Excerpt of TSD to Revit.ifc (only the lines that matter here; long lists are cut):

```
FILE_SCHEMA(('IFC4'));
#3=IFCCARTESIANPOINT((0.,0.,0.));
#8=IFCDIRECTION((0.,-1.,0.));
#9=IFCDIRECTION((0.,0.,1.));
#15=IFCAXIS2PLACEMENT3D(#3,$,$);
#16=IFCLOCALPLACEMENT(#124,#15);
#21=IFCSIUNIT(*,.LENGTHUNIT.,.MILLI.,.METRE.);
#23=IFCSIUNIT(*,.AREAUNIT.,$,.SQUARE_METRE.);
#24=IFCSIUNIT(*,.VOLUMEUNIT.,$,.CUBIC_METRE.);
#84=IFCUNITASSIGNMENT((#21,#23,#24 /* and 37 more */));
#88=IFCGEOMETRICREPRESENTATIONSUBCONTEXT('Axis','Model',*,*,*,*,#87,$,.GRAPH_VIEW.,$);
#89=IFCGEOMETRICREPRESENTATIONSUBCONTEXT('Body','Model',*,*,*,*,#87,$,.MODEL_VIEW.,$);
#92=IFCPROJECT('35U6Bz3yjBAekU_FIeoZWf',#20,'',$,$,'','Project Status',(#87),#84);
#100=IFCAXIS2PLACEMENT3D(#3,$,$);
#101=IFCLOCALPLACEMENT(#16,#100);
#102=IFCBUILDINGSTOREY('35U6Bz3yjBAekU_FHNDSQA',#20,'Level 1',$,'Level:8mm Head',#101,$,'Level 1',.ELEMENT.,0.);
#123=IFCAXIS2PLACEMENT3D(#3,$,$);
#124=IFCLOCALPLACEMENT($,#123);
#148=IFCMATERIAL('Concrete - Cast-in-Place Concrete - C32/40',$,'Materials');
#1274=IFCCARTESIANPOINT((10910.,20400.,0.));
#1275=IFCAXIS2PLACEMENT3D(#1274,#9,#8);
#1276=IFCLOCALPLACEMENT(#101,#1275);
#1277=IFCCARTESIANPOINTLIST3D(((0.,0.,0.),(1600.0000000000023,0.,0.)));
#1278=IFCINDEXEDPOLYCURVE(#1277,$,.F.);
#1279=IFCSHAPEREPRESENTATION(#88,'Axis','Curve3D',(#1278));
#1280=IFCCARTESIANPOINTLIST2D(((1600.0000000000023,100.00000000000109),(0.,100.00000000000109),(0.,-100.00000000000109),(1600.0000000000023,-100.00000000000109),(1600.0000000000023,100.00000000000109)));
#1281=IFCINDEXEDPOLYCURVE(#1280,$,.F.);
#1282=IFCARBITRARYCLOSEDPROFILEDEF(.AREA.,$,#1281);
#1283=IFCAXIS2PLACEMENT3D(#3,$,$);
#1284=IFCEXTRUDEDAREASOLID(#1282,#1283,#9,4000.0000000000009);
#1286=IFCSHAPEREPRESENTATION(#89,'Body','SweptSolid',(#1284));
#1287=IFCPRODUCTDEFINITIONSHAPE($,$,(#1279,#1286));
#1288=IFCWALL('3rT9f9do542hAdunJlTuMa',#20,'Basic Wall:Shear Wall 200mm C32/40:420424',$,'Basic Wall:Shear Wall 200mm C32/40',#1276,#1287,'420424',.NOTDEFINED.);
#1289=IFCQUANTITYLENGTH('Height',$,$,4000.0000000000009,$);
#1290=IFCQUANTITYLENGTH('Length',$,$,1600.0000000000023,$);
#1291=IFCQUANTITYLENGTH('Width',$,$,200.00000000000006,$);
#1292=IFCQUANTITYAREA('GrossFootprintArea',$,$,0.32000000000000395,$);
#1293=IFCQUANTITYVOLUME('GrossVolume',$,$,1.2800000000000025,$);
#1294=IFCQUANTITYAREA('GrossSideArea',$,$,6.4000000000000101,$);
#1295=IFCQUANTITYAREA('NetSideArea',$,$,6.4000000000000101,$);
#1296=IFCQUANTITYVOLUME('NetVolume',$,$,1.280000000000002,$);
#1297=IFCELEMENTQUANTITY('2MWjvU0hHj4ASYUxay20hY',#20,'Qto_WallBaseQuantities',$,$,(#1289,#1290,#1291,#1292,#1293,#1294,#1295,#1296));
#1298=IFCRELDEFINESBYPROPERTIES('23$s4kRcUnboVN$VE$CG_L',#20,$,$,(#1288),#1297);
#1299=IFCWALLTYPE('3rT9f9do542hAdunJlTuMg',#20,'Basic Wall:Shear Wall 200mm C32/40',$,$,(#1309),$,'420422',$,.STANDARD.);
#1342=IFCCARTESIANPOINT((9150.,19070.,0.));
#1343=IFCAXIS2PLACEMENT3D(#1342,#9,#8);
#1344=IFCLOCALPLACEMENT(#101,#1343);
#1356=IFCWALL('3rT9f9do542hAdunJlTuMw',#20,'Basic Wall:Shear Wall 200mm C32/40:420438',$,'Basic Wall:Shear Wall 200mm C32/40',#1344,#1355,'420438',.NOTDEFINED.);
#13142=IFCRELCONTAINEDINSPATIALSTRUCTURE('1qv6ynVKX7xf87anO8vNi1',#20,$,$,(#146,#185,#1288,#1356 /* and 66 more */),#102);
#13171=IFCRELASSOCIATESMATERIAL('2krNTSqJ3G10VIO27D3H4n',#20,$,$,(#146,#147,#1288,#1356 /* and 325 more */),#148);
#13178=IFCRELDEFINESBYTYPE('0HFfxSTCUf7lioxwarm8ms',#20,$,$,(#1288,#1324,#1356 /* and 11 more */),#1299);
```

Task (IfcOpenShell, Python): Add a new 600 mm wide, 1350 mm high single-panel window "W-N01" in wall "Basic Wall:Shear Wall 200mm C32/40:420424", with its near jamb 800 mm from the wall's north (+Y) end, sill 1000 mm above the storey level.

```python
import numpy as np
import ifcopenshell
import ifcopenshell.api.feature
import ifcopenshell.api.geometry
import ifcopenshell.api.pset
import ifcopenshell.api.root
import ifcopenshell.api.spatial
import ifcopenshell.geom
import ifcopenshell.util.element
import ifcopenshell.util.placement
import ifcopenshell.util.representation
import ifcopenshell.util.shape
import ifcopenshell.util.unit

model = ifcopenshell.open("TSD to Revit.ifc")
unit_scale = ifcopenshell.util.unit.calculate_unit_scale(model)
area_scale = ifcopenshell.util.unit.calculate_unit_scale(model, "AREAUNIT")
volume_scale = ifcopenshell.util.unit.calculate_unit_scale(model, "VOLUMEUNIT")
settings = ifcopenshell.geom.settings()


def volume(element):
    """Net volume in cubic metres, openings subtracted."""
    shape = ifcopenshell.geom.create_shape(settings, element)
    return ifcopenshell.util.shape.get_volume(shape.geometry)


wall = model.by_guid("3rT9f9do542hAdunJlTuMa")
storey = ifcopenshell.util.element.get_container(wall, ifc_class="IfcBuildingStorey")
context = ifcopenshell.util.representation.get_context(model, "Model", "Body", "MODEL_VIEW")
before = volume(wall)

width, height, from_end, sill = 0.6, 1.35, 0.8, 1  # metres

# The wall runs along its own X axis, and the end named is its -X end.
wall_shape = ifcopenshell.geom.create_shape(settings, wall)
x, y, z = ifcopenshell.util.shape.get_vertices(wall_shape.geometry).T
start = x.min() + from_end
face, thickness = float(y.min()), float(y.max() - y.min())
wall_matrix = ifcopenshell.util.placement.get_local_placement(wall.ObjectPlacement)
level = ifcopenshell.util.placement.get_local_placement(storey.ObjectPlacement)[2, 3]


def in_wall(x, y):
    """Placement at x, y metres in the wall's axes, at sill height."""
    matrix = wall_matrix.copy()
    matrix[:, 3] = wall_matrix @ np.array([x / unit_scale, y / unit_scale, 0.0, 1.0])
    matrix[2, 3] = level + sill / unit_scale
    return matrix


# Opening: a box that overshoots both wall faces by 50 mm.
opening = ifcopenshell.api.root.create_entity(model, ifc_class="IfcOpeningElement", predefined_type="OPENING")
box = ifcopenshell.api.geometry.add_wall_representation(
    model, context=context, length=width, height=height, thickness=thickness + 0.1
)
ifcopenshell.api.geometry.assign_representation(model, product=opening, representation=box)
ifcopenshell.api.geometry.edit_object_placement(model, product=opening, matrix=in_wall(start, face - 0.05), is_si=False)
ifcopenshell.api.feature.add_feature(model, feature=opening, element=wall)

window = ifcopenshell.api.root.create_entity(model, ifc_class="IfcWindow", name="W-N01", predefined_type="WINDOW")
window.OverallWidth, window.OverallHeight = width / unit_scale, height / unit_scale
window.PartitioningType = "SINGLE_PANEL"
body = ifcopenshell.api.geometry.add_window_representation(
    model,
    context=context,
    overall_width=window.OverallWidth,
    overall_height=window.OverallHeight,
    partition_type="SINGLE_PANEL",
)
ifcopenshell.api.geometry.assign_representation(model, product=window, representation=body)
ifcopenshell.api.spatial.assign_container(model, products=[window], relating_structure=storey)
ifcopenshell.api.feature.add_filling(model, opening=opening, element=window)

# Centre the window in the wall's thickness.
ifcopenshell.api.geometry.edit_object_placement(model, product=window, matrix=in_wall(start, face), is_si=False)
window_shape = ifcopenshell.geom.create_shape(settings, window)
depth = ifcopenshell.util.shape.get_vertices(window_shape.geometry)[:, 1]
offset = face + thickness / 2 - (depth.min() + depth.max()) / 2
ifcopenshell.api.geometry.edit_object_placement(model, product=window, matrix=in_wall(start, offset), is_si=False)

after = volume(wall)

# Update the wall's stored quantities.
qto = model.by_id(ifcopenshell.util.element.get_pset(wall, "Qto_WallBaseQuantities", should_inherit=False)["id"])
ifcopenshell.api.pset.edit_qto(model, qto=qto, properties={
    "NetSideArea": after / thickness / area_scale,
    "NetVolume": after / volume_scale,
})

print(f"wall volume {before:.3f} -> {after:.3f} m3")

model.write("TSD to Revit_edited.ifc")
```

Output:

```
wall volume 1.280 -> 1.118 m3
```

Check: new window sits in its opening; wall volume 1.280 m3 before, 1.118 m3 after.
